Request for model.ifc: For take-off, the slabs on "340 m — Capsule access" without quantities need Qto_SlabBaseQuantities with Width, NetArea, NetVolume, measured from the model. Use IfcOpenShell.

First a look at what the model holds.

```python
import ifcopenshell
import ifcopenshell.util.element
import ifcopenshell.util.unit

model = ifcopenshell.open("model.ifc")
print(model.schema)
for unit_type in ("LENGTHUNIT", "AREAUNIT", "VOLUMEUNIT"):
    print(unit_type, ifcopenshell.util.unit.calculate_unit_scale(model, unit_type))
storey = next(s for s in model.by_type("IfcBuildingStorey") if s.Name == "340 m — Capsule access")
slabs = [e for e in ifcopenshell.util.element.get_decomposition(storey) if e.is_a("IfcSlab")]
for e in sorted(slabs, key=lambda e: e.id()):
    print(e.id(), e.is_a(), e.Name, list(ifcopenshell.util.element.get_psets(e, qtos_only=True)), sep=" | ")
```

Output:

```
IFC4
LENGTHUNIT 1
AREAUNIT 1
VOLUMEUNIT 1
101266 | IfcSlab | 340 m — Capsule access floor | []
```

```python
import ifcopenshell
import ifcopenshell.api.pset
import ifcopenshell.geom
import ifcopenshell.util.element
import ifcopenshell.util.shape
import ifcopenshell.util.unit

model = ifcopenshell.open("model.ifc")
unit_scale = ifcopenshell.util.unit.calculate_unit_scale(model)
area_scale = ifcopenshell.util.unit.calculate_unit_scale(model, "AREAUNIT")
volume_scale = ifcopenshell.util.unit.calculate_unit_scale(model, "VOLUMEUNIT")
settings = ifcopenshell.geom.settings()

storey = next(s for s in model.by_type("IfcBuildingStorey") if s.Name == "340 m — Capsule access")
slabs = [e for e in ifcopenshell.util.element.get_decomposition(storey) if e.is_a("IfcSlab")]

for e in sorted(slabs, key=lambda e: e.id()):
    if ifcopenshell.util.element.get_psets(e, qtos_only=True, should_inherit=False):
        continue
    # Geometry comes back in metres, in the element's own axes.
    shape = ifcopenshell.geom.create_shape(settings, e)
    values = {
        "Width": ifcopenshell.util.shape.get_z(shape.geometry) / unit_scale,
        "NetArea": ifcopenshell.util.shape.get_footprint_area(shape.geometry) / area_scale,
        "NetVolume": ifcopenshell.util.shape.get_volume(shape.geometry) / volume_scale,
    }
    qto = ifcopenshell.api.pset.add_qto(model, product=e, name="Qto_SlabBaseQuantities")
    ifcopenshell.api.pset.edit_qto(model, qto=qto, properties=values)
    print(e.id(), {k: round(v, 3) for k, v in values.items()})

model.write("model-out.ifc")
```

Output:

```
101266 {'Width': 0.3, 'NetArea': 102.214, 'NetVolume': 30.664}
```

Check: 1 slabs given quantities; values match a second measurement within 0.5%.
